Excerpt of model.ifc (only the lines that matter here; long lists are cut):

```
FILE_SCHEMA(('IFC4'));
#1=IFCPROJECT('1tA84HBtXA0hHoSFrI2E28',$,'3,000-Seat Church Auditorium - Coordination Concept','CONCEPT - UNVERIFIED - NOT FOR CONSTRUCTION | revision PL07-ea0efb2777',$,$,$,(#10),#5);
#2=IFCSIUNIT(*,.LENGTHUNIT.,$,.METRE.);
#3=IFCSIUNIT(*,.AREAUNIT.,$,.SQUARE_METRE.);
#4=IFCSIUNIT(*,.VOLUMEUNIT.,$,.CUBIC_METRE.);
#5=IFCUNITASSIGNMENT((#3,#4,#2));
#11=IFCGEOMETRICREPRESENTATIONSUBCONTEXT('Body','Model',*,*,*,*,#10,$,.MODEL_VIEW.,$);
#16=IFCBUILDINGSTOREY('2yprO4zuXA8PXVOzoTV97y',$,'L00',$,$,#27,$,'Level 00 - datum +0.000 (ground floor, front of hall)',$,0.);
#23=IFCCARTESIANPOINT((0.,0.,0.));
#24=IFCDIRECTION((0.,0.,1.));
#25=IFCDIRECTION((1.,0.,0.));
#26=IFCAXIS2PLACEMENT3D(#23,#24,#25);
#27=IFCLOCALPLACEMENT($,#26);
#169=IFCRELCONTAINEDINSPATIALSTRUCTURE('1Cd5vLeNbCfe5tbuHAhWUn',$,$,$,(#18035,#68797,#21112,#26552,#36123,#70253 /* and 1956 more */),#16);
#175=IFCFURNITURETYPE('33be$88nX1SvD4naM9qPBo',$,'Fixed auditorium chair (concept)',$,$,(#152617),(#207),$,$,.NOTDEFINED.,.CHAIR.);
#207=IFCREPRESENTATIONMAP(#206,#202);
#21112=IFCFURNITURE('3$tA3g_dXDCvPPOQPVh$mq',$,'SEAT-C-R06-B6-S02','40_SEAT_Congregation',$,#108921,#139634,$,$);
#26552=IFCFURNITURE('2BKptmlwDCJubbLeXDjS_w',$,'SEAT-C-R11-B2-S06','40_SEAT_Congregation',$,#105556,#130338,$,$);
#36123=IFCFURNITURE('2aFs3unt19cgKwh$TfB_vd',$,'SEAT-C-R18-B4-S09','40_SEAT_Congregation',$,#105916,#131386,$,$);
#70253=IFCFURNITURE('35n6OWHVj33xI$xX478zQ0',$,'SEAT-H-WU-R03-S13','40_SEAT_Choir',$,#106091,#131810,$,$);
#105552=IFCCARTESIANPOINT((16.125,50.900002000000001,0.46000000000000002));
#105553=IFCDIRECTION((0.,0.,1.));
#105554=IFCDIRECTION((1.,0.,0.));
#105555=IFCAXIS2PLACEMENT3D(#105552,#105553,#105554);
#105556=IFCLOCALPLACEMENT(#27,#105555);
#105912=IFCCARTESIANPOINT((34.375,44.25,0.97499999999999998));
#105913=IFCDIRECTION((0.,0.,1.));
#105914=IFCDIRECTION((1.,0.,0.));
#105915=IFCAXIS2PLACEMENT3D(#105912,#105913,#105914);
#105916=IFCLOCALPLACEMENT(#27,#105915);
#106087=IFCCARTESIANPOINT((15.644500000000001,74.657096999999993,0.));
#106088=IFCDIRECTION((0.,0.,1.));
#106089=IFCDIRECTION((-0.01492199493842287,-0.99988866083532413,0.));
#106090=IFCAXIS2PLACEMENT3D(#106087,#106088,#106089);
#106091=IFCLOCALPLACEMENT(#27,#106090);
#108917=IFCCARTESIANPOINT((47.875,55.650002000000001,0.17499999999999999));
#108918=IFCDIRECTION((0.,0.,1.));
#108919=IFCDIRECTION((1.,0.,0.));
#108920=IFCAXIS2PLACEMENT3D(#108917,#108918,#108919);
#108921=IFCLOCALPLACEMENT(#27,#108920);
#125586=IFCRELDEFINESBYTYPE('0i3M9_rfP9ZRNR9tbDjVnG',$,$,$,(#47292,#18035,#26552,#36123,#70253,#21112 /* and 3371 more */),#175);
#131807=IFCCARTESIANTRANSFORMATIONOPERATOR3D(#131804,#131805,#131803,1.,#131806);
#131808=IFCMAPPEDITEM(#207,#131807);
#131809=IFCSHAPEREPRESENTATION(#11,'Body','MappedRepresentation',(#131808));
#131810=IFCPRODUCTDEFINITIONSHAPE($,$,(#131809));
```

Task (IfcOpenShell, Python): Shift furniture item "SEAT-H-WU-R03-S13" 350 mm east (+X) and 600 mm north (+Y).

```python
import ifcopenshell
import ifcopenshell.api.geometry
import ifcopenshell.util.placement

model = ifcopenshell.open("model.ifc")

item = model.by_guid("35n6OWHVj33xI$xX478zQ0")
matrix = ifcopenshell.util.placement.get_local_placement(item.ObjectPlacement)
matrix[0, 3] += 0.35
matrix[1, 3] += 0.6
ifcopenshell.api.geometry.edit_object_placement(model, product=item, matrix=matrix, is_si=False)

print(ifcopenshell.util.placement.get_local_placement(item.ObjectPlacement).round(3) + 0.0)

model.write("model_v2.ifc")
```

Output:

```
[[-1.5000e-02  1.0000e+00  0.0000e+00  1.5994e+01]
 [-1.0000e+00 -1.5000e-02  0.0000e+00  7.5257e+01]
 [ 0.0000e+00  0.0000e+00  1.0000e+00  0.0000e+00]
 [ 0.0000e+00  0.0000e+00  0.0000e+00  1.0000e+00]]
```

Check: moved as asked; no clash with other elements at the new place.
